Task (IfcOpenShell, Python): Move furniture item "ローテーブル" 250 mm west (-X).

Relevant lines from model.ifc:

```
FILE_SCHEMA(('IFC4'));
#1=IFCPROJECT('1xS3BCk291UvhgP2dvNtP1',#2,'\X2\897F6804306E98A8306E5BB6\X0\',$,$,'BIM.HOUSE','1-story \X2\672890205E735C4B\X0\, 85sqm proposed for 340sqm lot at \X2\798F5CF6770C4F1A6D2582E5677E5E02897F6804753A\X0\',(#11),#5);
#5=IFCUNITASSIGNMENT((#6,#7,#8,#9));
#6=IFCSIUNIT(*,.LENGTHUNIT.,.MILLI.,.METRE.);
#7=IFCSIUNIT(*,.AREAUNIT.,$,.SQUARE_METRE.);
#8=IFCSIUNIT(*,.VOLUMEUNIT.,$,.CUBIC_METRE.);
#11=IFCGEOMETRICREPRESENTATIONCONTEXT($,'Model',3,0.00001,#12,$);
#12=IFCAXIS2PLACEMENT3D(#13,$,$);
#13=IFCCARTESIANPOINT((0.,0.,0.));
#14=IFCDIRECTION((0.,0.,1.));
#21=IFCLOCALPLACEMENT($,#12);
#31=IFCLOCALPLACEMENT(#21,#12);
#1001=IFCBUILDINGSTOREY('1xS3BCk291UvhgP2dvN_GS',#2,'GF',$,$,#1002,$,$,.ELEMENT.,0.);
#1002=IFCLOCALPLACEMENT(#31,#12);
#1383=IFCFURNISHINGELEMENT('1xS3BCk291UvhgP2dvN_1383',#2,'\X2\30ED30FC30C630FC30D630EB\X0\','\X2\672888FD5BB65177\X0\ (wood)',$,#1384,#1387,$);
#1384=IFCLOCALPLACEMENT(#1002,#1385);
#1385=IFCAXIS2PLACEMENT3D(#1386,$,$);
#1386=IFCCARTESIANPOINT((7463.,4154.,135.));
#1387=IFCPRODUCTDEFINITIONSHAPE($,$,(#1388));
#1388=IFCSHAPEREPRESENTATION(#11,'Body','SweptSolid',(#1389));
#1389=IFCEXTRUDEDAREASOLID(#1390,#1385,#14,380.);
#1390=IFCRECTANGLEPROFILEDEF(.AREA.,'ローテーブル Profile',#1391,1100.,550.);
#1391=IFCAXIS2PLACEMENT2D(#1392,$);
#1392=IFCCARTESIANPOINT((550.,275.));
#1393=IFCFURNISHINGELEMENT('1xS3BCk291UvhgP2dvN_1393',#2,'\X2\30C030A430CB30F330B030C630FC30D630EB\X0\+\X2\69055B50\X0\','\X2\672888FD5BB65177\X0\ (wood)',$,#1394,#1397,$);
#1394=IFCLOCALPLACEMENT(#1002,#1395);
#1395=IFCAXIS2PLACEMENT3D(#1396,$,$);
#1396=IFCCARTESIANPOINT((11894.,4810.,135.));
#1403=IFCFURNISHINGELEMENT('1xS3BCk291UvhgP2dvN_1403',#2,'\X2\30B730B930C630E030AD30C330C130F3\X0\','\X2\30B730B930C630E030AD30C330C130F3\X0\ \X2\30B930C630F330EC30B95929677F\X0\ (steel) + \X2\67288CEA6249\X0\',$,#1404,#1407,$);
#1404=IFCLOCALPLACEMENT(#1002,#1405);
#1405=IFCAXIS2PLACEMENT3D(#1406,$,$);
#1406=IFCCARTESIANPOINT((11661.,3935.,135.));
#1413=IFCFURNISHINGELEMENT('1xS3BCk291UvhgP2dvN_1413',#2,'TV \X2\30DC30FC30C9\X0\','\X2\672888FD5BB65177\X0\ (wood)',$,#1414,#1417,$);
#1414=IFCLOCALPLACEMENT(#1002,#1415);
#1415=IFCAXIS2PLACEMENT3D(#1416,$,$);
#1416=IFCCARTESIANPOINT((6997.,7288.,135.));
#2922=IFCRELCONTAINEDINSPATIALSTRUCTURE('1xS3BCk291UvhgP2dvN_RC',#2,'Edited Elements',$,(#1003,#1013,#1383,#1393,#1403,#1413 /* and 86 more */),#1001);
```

```python
import ifcopenshell
import ifcopenshell.api.geometry
import ifcopenshell.util.placement
import ifcopenshell.util.unit

model = ifcopenshell.open("model.ifc")
unit_scale = ifcopenshell.util.unit.calculate_unit_scale(model)

item = model.by_id(1383)
matrix = ifcopenshell.util.placement.get_local_placement(item.ObjectPlacement)
matrix[0, 3] -= 0.25 / unit_scale
ifcopenshell.api.geometry.edit_object_placement(model, product=item, matrix=matrix, is_si=False)

print(ifcopenshell.util.placement.get_local_placement(item.ObjectPlacement).round(3) + 0.0)

model.write("model_updated.ifc")
```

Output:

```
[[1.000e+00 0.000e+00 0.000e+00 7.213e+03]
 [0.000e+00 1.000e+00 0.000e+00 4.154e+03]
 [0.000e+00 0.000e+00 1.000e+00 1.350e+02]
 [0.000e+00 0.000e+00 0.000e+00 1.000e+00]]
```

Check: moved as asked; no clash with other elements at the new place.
